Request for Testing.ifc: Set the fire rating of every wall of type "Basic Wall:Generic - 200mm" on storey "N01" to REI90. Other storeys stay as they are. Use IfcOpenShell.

First a look at what the model holds.

```python
import ifcopenshell
import ifcopenshell.util.element

model = ifcopenshell.open("Testing.ifc")
print(model.schema)
storey = next(s for s in model.by_type("IfcBuildingStorey") if s.Name == "N01")
walls = [e for e in ifcopenshell.util.element.get_decomposition(storey) if e.is_a("IfcWall")]
seen = {}
for e in walls:
    element_type = ifcopenshell.util.element.get_type(e)
    key = (element_type.Name if element_type != e and element_type else None, ifcopenshell.util.element.get_pset(e, "Pset_WallCommon", "FireRating"))
    seen[key] = seen.get(key, 0) + 1
for (name, value), count in sorted(seen.items(), key=str):
    print(count, "x", name, "|", value)
```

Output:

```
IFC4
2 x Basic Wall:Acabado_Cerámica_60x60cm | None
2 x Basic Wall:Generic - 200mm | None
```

```python
import ifcopenshell
import ifcopenshell.api.pset
import ifcopenshell.util.element

model = ifcopenshell.open("Testing.ifc")

storey = next(s for s in model.by_type("IfcBuildingStorey") if s.Name == "N01")
walls = [e for e in ifcopenshell.util.element.get_decomposition(storey) if e.is_a("IfcWall")]

count = 0
for e in walls:
    element_type = ifcopenshell.util.element.get_type(e)
    if element_type in (None, e) or element_type.Name != "Basic Wall:Generic - 200mm":
        continue
    # add_pset returns the element's existing set when there is one.
    pset = ifcopenshell.api.pset.add_pset(model, product=e, name="Pset_WallCommon")
    ifcopenshell.api.pset.edit_pset(model, pset=pset, properties={"FireRating": "REI90"})
    count += 1

print(count, "walls updated")

model.write("Testing-out.ifc")
```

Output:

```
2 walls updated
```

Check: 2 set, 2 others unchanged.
